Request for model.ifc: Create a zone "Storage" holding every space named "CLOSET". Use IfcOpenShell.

First a look at what the model holds.

```python
import ifcopenshell

model = ifcopenshell.open("model.ifc")
print(model.schema)
seen = {}
for space in model.by_type("IfcSpace"):
    seen[space.LongName] = seen.get(space.LongName, 0) + 1
for name, count in sorted(seen.items(), key=str):
    print(count, "x", name)
print("zones:", [z.Name for z in model.by_type("IfcZone")][:20])
```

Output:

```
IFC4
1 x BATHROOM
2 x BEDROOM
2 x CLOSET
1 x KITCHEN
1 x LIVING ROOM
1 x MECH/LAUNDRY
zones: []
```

```python
import ifcopenshell
import ifcopenshell.api.group
import ifcopenshell.api.root

model = ifcopenshell.open("model.ifc")

names = {"CLOSET"}
spaces = [s for s in model.by_type("IfcSpace") if s.LongName in names]

zone = ifcopenshell.api.root.create_entity(model, ifc_class="IfcZone", name="Storage")
ifcopenshell.api.group.assign_group(model, products=spaces, group=zone)
print(len(spaces), "spaces in", zone.Name)

model.write("model_updated.ifc")
```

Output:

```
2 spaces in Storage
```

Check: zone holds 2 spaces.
